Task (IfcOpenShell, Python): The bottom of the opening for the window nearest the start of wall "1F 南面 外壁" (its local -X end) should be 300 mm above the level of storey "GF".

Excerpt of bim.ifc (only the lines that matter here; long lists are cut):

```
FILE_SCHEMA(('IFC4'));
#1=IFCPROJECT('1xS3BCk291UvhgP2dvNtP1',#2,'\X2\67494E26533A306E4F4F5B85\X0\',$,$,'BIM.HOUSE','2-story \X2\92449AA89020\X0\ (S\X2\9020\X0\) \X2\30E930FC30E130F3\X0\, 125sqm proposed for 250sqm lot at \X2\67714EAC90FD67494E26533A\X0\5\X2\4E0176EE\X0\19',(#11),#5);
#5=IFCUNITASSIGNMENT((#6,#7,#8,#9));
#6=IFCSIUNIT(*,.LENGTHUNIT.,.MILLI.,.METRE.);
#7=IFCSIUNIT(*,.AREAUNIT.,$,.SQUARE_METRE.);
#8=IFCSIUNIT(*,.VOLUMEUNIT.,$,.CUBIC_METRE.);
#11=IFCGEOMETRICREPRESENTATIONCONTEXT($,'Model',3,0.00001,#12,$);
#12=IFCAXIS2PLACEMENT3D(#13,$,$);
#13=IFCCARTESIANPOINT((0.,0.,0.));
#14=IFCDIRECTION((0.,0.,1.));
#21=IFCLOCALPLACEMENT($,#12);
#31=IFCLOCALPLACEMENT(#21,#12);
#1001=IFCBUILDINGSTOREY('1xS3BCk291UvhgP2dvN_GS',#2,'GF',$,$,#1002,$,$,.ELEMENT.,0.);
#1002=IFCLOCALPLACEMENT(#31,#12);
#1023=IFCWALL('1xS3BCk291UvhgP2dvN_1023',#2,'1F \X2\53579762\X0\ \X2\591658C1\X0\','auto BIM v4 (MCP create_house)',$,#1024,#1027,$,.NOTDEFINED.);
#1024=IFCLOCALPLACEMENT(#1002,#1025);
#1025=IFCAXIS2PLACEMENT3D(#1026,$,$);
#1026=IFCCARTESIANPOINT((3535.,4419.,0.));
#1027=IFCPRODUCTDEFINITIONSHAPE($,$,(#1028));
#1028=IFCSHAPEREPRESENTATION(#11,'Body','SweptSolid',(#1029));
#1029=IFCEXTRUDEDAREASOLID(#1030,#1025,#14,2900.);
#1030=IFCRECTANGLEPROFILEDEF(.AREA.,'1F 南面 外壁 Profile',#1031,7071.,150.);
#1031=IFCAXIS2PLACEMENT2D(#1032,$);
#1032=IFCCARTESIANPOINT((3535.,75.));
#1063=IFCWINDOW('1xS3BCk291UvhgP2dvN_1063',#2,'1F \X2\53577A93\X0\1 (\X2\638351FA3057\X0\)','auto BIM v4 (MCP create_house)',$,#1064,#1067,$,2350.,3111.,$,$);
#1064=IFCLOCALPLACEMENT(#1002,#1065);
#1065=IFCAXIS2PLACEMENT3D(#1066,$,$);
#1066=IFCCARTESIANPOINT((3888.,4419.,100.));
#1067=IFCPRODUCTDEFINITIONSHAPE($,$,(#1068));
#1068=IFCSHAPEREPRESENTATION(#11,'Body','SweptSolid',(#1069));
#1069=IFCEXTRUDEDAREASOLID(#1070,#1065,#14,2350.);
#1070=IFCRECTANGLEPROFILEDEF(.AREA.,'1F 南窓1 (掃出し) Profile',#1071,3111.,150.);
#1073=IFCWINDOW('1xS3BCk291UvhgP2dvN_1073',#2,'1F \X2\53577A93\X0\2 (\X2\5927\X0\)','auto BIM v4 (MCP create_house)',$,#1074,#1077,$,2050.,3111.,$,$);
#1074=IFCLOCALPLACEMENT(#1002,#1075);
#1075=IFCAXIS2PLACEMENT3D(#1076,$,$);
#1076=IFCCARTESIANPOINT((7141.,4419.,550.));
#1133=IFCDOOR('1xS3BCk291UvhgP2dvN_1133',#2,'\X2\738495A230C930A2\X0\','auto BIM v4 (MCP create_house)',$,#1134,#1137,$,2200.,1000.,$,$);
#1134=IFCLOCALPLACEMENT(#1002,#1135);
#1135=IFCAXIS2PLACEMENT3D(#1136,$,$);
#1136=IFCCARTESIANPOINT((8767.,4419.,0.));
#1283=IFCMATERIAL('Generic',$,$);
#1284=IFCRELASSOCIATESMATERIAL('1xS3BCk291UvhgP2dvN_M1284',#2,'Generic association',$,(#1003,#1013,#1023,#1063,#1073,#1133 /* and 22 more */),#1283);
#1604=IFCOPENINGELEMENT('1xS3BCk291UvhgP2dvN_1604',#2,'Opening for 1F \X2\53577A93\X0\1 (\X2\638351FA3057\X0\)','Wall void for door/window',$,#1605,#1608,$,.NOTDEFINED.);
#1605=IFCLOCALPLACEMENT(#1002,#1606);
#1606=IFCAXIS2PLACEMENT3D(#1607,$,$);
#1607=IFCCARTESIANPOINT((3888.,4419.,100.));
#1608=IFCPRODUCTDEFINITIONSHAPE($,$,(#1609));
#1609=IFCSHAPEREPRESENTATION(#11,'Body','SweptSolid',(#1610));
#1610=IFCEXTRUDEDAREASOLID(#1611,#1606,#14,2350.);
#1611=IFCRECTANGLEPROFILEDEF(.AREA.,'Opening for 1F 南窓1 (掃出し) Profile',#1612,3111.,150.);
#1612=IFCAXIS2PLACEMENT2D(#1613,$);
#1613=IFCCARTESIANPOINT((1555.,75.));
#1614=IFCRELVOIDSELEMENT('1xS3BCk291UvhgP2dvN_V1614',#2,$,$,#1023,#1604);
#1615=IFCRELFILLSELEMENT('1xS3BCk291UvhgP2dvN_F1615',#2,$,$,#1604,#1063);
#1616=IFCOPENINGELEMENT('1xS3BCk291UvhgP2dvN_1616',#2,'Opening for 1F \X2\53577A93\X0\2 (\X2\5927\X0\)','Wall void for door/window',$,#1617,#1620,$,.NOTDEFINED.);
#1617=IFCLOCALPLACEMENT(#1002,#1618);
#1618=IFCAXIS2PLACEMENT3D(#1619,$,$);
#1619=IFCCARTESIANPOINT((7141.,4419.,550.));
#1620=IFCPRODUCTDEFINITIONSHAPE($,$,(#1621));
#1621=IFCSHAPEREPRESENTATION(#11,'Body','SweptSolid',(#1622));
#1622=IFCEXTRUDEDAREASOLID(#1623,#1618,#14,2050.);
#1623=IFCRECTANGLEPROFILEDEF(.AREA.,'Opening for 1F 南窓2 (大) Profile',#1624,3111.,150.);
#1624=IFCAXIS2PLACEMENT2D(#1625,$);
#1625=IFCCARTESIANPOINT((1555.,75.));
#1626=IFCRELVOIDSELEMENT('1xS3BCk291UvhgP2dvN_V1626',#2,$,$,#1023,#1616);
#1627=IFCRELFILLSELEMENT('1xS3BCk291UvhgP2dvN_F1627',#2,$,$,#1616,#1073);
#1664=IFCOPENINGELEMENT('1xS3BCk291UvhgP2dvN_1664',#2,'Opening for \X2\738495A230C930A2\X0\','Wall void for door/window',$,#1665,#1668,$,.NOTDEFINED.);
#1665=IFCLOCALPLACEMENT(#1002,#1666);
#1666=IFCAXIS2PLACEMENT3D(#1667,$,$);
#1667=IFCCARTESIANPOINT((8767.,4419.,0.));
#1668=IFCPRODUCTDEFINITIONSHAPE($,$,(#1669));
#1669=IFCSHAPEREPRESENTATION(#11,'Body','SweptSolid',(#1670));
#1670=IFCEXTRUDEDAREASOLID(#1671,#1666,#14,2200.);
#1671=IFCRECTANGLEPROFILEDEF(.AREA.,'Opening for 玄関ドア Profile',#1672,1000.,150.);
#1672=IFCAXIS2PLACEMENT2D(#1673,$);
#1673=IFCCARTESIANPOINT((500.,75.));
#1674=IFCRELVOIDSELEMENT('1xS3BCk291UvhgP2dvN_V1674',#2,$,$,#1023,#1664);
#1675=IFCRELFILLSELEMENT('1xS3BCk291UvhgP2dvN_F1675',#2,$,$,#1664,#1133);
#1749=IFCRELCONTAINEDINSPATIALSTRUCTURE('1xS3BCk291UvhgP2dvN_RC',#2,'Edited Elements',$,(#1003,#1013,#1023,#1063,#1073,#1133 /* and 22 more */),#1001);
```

```python
import numpy as np
import ifcopenshell
import ifcopenshell.api.geometry
import ifcopenshell.geom
import ifcopenshell.util.element
import ifcopenshell.util.placement
import ifcopenshell.util.shape
import ifcopenshell.util.unit

model = ifcopenshell.open("bim.ifc")
unit_scale = ifcopenshell.util.unit.calculate_unit_scale(model)

window = model.by_guid("1xS3BCk291UvhgP2dvN_1063")
opening = window.FillsVoids[0].RelatingOpeningElement
storey = ifcopenshell.util.element.get_container(window, ifc_class="IfcBuildingStorey")
level = ifcopenshell.util.placement.get_local_placement(storey.ObjectPlacement)[2, 3]

# The opening's origin need not be at the sill, so measure its lowest point.
shape = ifcopenshell.geom.create_shape(ifcopenshell.geom.settings(), opening)
bottom = ifcopenshell.util.shape.get_shape_bottom_elevation(shape, shape.geometry) / unit_scale
dz = level + 0.3 / unit_scale - bottom

shift = np.array([0.0, 0.0, dz])
# The window is not placed relative to its opening, so move both.
for product in (opening, window):
    matrix = ifcopenshell.util.placement.get_local_placement(product.ObjectPlacement)
    matrix[:3, 3] += shift
    ifcopenshell.api.geometry.edit_object_placement(model, product=product, matrix=matrix, is_si=False)

print(f"moved by {dz * unit_scale:+.3f} m")

model.write("bim_rev.ifc")
```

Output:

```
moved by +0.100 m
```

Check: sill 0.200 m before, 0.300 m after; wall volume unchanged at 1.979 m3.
